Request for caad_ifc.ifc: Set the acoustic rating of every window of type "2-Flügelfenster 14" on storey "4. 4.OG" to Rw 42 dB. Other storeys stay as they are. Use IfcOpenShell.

First a look at what the model holds.

```python
import ifcopenshell
import ifcopenshell.util.element

model = ifcopenshell.open("caad_ifc.ifc")
print(model.schema)
storey = next(s for s in model.by_type("IfcBuildingStorey") if s.Name == "4. 4.OG")
windows = [e for e in ifcopenshell.util.element.get_decomposition(storey) if e.is_a("IfcWindow")]
seen = {}
for e in windows:
    element_type = ifcopenshell.util.element.get_type(e)
    key = (element_type.Name if element_type != e and element_type else None, ifcopenshell.util.element.get_pset(e, "Pset_WindowCommon", "AcousticRating"))
    seen[key] = seen.get(key, 0) + 1
for (name, value), count in sorted(seen.items(), key=str):
    print(count, "x", name, "|", value)
```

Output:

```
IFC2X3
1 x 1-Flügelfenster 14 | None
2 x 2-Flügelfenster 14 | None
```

```python
import ifcopenshell
import ifcopenshell.api.pset
import ifcopenshell.util.element

model = ifcopenshell.open("caad_ifc.ifc")

storey = next(s for s in model.by_type("IfcBuildingStorey") if s.Name == "4. 4.OG")
windows = [e for e in ifcopenshell.util.element.get_decomposition(storey) if e.is_a("IfcWindow")]

count = 0
for e in windows:
    element_type = ifcopenshell.util.element.get_type(e)
    if element_type in (None, e) or element_type.Name != "2-Flügelfenster 14":
        continue
    # add_pset returns the element's existing set when there is one.
    pset = ifcopenshell.api.pset.add_pset(model, product=e, name="Pset_WindowCommon")
    ifcopenshell.api.pset.edit_pset(model, pset=pset, properties={"AcousticRating": "Rw 42 dB"})
    count += 1

print(count, "windows updated")

model.write("caad_ifc_rev.ifc")
```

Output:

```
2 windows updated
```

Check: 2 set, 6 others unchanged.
